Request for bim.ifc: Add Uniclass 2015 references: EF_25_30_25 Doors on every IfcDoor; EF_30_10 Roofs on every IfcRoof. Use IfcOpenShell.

First a look at what the model holds.

```python
import ifcopenshell

model = ifcopenshell.open("bim.ifc")
print(model.schema)
print("classifications:", [c.Name for c in model.by_type("IfcClassification")])
for ifc_class in ("IfcDoor", "IfcRoof", "IfcStair", "IfcWall", "IfcWindow"):
    print(ifc_class, len(model.by_type(ifc_class)))
```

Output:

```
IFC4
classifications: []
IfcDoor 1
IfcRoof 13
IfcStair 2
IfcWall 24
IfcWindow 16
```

```python
import ifcopenshell
import ifcopenshell.api.classification

model = ifcopenshell.open("bim.ifc")

system = ifcopenshell.api.classification.add_classification(model, classification="Uniclass 2015")

codes = {
    "IfcDoor": ("EF_25_30_25", "Doors"),
    "IfcRoof": ("EF_30_10", "Roofs"),
}
for ifc_class, (code, name) in codes.items():
    products = model.by_type(ifc_class)
    ifcopenshell.api.classification.add_reference(
        model, products=products, classification=system, identification=code, name=name
    )
    print(code, len(products))

model.write("bim_v2.ifc")
```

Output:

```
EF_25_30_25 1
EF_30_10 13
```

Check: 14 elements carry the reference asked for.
